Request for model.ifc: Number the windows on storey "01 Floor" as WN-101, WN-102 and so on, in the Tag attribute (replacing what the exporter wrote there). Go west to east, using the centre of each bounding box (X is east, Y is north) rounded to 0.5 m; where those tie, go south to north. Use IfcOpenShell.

First a look at what the model holds.

```python
import ifcopenshell
import ifcopenshell.util.element
import ifcopenshell.util.placement

model = ifcopenshell.open("model.ifc")
print(model.schema)
storey = next(s for s in model.by_type("IfcBuildingStorey") if s.Name == "01 Floor")
windows = [e for e in ifcopenshell.util.element.get_decomposition(storey) if e.is_a("IfcWindow")]
for e in sorted(windows, key=lambda e: e.id()):
    origin = ifcopenshell.util.placement.get_local_placement(e.ObjectPlacement)[:3, 3]
    print(e.id(), e.Tag, e.Name, origin.round(2) + 0.0, sep=" | ")
```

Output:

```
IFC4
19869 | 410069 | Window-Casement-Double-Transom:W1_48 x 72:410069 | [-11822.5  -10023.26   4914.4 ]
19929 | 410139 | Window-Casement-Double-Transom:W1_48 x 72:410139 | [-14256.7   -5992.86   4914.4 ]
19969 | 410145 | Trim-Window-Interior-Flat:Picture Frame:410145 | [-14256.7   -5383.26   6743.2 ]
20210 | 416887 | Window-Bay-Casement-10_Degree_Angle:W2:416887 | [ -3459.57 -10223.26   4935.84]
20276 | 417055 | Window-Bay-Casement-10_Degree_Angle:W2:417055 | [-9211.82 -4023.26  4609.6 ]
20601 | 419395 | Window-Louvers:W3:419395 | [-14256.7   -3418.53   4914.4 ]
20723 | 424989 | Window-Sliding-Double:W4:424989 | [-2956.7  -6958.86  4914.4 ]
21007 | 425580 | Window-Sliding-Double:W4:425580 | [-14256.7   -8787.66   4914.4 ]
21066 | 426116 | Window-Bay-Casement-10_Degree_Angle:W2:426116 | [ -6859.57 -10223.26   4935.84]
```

```python
import ifcopenshell
import ifcopenshell.geom
import ifcopenshell.util.element
import ifcopenshell.util.shape

model = ifcopenshell.open("model.ifc")
settings = ifcopenshell.geom.settings()
settings.set("use-world-coords", True)


def centre(element):
    shape = ifcopenshell.geom.create_shape(settings, element)
    return ifcopenshell.util.shape.get_bbox_centroid(shape.geometry)


storey = next(s for s in model.by_type("IfcBuildingStorey") if s.Name == "01 Floor")
windows = [e for e in ifcopenshell.util.element.get_decomposition(storey) if e.is_a("IfcWindow")]

# Insertion points can sit at a corner or the storey origin, so sort by the geometry (in metres).
centres = {e: centre(e) for e in windows}
windows.sort(key=lambda e: (round(centres[e][0] / 0.5), centres[e][1]))

for i, e in enumerate(windows, start=1):
    number = f"WN-1{i:02d}"
    e.Tag = number
    print(e.id(), number)

model.write("model_v2.ifc")
```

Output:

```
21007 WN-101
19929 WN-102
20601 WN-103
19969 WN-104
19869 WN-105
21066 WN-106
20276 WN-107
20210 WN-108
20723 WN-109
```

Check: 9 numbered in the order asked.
